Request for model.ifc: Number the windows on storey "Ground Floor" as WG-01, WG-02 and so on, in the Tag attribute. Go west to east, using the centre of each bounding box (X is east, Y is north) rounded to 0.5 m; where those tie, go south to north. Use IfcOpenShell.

First a look at what the model holds.

```python
import ifcopenshell
import ifcopenshell.util.element
import ifcopenshell.util.placement

model = ifcopenshell.open("model.ifc")
print(model.schema)
storey = next(s for s in model.by_type("IfcBuildingStorey") if s.Name == "Ground Floor")
windows = [e for e in ifcopenshell.util.element.get_decomposition(storey) if e.is_a("IfcWindow")]
for e in sorted(windows, key=lambda e: e.id()):
    origin = ifcopenshell.util.placement.get_local_placement(e.ObjectPlacement)[:3, 3]
    print(e.id(), e.Tag, e.Name, origin.round(2) + 0.0, sep=" | ")
```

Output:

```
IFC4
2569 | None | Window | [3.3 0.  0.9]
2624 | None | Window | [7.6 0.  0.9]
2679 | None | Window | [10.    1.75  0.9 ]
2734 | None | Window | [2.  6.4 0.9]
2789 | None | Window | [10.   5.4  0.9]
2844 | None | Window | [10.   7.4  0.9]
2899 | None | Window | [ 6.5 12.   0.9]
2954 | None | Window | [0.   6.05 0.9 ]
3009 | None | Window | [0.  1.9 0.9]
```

```python
import ifcopenshell
import ifcopenshell.geom
import ifcopenshell.util.element
import ifcopenshell.util.shape

model = ifcopenshell.open("model.ifc")
settings = ifcopenshell.geom.settings()
settings.set("use-world-coords", True)


def centre(element):
    shape = ifcopenshell.geom.create_shape(settings, element)
    return ifcopenshell.util.shape.get_bbox_centroid(shape.geometry)


storey = next(s for s in model.by_type("IfcBuildingStorey") if s.Name == "Ground Floor")
windows = [e for e in ifcopenshell.util.element.get_decomposition(storey) if e.is_a("IfcWindow")]

# Insertion points can sit at a corner or the storey origin, so sort by the geometry (in metres).
centres = {e: centre(e) for e in windows}
windows.sort(key=lambda e: (round(centres[e][0] / 0.5), centres[e][1]))

for i, e in enumerate(windows, start=1):
    number = f"WG-{i:02d}"
    e.Tag = number
    print(e.id(), number)

model.write("model_edited.ifc")
```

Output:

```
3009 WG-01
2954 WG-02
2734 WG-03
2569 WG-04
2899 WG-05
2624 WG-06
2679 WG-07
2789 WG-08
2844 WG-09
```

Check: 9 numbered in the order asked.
